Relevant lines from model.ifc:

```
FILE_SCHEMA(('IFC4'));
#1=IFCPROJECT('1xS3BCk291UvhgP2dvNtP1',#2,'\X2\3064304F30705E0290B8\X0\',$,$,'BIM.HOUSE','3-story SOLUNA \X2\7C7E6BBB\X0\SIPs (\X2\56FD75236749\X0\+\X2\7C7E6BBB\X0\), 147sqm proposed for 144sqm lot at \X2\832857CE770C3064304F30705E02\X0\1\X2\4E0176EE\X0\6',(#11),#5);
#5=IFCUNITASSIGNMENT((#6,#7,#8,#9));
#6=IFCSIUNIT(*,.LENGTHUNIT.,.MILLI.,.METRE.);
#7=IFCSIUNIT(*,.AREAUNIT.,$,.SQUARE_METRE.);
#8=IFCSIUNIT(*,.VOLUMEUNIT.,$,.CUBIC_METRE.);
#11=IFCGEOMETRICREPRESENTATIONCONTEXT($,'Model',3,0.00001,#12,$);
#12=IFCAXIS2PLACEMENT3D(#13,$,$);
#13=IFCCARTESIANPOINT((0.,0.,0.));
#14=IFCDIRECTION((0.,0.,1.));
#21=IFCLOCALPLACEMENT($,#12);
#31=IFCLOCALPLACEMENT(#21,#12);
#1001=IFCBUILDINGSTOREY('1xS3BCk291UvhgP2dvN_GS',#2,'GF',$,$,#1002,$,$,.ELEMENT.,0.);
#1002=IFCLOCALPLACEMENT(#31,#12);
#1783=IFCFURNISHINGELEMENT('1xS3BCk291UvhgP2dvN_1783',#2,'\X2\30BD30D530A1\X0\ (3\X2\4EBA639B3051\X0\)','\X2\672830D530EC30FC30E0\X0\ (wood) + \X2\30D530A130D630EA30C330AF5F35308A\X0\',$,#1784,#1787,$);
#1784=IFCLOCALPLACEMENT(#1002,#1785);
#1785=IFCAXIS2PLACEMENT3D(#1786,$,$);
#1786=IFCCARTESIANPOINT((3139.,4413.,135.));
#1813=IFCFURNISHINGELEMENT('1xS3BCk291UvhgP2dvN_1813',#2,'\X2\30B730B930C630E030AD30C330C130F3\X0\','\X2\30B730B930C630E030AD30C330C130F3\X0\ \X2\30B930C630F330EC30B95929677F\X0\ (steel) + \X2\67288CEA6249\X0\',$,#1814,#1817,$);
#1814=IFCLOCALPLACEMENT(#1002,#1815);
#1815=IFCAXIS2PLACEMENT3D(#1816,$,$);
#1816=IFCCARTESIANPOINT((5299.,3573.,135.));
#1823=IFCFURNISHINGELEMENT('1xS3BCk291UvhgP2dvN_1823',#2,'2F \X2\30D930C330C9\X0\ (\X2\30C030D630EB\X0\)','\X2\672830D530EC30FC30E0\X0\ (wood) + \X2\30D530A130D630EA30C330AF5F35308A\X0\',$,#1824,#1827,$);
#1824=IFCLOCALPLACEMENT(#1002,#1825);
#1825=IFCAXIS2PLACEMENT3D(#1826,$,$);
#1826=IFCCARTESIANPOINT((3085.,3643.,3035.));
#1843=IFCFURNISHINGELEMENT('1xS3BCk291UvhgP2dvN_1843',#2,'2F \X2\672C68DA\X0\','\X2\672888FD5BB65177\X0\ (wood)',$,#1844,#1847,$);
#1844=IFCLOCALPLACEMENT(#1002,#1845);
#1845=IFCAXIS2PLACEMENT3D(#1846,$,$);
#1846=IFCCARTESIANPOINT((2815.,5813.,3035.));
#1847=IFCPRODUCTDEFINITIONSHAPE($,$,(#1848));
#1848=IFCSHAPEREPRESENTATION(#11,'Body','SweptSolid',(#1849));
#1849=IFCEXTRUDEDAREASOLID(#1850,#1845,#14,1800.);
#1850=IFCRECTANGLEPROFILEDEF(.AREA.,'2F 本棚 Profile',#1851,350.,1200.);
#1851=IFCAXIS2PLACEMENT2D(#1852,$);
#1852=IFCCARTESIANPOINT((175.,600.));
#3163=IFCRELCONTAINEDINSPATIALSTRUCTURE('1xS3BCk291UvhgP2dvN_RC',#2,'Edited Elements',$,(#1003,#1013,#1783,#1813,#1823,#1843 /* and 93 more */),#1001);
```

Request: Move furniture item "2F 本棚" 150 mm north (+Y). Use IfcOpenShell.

```python
import ifcopenshell
import ifcopenshell.api.geometry
import ifcopenshell.util.placement
import ifcopenshell.util.unit

model = ifcopenshell.open("model.ifc")
unit_scale = ifcopenshell.util.unit.calculate_unit_scale(model)

item = model.by_guid("1xS3BCk291UvhgP2dvN_1843")
matrix = ifcopenshell.util.placement.get_local_placement(item.ObjectPlacement)
matrix[1, 3] += 0.15 / unit_scale
ifcopenshell.api.geometry.edit_object_placement(model, product=item, matrix=matrix, is_si=False)

print(ifcopenshell.util.placement.get_local_placement(item.ObjectPlacement).round(3) + 0.0)

model.write("model-out.ifc")
```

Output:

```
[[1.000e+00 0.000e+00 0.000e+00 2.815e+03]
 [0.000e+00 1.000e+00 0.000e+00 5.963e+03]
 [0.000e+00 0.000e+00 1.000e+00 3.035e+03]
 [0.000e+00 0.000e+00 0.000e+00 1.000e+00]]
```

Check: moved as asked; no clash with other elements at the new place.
